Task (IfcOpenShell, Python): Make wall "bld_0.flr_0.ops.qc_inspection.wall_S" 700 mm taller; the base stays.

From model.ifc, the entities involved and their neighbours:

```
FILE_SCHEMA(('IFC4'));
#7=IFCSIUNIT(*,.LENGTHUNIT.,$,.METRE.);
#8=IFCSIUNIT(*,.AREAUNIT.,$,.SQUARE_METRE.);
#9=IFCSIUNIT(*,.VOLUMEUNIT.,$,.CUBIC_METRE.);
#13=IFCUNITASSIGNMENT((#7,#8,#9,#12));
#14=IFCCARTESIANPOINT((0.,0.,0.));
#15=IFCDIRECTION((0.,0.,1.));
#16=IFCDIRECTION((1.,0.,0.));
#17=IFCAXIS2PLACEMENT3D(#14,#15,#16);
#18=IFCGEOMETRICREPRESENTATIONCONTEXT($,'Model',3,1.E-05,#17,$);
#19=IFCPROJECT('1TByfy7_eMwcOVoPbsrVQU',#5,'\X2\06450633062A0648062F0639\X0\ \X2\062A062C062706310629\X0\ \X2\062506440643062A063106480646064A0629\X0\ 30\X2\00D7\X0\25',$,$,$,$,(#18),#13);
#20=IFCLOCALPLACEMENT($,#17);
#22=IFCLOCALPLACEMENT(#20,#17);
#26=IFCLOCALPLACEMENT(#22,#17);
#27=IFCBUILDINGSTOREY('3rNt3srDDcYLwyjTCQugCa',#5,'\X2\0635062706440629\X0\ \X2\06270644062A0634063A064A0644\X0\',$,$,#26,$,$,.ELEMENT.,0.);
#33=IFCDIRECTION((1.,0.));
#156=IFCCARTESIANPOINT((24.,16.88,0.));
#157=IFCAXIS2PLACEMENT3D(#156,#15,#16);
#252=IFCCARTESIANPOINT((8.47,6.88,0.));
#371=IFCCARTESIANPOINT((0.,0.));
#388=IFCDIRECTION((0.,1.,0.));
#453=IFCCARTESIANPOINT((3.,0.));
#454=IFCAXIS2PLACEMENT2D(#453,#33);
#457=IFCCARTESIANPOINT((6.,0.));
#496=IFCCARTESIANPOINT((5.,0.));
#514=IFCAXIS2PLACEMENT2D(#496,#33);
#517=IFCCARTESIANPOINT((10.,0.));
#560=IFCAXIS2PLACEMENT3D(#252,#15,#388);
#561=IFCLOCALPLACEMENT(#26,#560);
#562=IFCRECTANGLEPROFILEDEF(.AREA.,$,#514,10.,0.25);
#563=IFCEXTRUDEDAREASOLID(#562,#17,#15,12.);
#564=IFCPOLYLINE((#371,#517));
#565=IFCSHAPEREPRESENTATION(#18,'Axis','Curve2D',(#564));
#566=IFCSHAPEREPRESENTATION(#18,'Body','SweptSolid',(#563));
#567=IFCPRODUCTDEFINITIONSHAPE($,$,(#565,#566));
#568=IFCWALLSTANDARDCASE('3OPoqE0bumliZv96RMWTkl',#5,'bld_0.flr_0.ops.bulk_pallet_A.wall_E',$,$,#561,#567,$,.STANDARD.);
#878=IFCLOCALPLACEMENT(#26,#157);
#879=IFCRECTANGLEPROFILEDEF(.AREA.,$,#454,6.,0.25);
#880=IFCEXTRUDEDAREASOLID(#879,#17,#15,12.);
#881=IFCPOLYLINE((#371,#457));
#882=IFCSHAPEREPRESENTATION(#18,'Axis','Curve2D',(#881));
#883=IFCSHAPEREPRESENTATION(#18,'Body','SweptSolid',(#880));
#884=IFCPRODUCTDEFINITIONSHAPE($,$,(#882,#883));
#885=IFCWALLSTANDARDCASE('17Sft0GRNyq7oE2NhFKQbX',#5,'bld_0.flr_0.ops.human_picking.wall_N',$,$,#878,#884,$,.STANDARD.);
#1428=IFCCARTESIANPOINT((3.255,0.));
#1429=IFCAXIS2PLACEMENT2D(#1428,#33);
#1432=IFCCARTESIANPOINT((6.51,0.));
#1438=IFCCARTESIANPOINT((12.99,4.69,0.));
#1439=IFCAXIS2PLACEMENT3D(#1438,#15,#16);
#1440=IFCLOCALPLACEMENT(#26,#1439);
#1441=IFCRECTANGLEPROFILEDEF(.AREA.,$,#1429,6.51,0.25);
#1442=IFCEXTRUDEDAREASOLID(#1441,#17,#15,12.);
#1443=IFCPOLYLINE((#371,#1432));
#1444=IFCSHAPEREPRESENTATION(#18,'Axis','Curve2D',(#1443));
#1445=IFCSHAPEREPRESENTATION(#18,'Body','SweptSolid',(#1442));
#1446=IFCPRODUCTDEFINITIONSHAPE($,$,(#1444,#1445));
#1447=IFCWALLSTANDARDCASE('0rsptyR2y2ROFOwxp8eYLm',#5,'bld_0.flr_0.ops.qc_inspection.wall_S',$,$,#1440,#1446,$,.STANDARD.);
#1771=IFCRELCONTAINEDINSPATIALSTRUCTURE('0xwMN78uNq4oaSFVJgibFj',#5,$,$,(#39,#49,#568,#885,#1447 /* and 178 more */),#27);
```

```python
import ifcopenshell
import ifcopenshell.geom
import ifcopenshell.util.shape

model = ifcopenshell.open("model.ifc")
settings = ifcopenshell.geom.settings()


def volume(element):
    """Net volume in cubic metres, openings subtracted."""
    shape = ifcopenshell.geom.create_shape(settings, element)
    return ifcopenshell.util.shape.get_volume(shape.geometry)


wall = model.by_id(1447)
before = volume(wall)

body = next(r for r in wall.Representation.Representations if r.RepresentationIdentifier == "Body")
solid = body.Items[0]
old_height = solid.Depth
solid.Depth += 0.7
after = volume(wall)

print(f"height {old_height:g} -> {solid.Depth:g}, volume {before:.3f} -> {after:.3f} m3")

model.write("model_rev.ifc")
```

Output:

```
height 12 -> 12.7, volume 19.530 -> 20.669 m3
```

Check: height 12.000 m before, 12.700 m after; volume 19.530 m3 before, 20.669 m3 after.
